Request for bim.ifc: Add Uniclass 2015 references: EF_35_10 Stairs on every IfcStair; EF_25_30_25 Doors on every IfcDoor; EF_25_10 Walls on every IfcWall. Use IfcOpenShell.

First a look at what the model holds.

```python
import ifcopenshell

model = ifcopenshell.open("bim.ifc")
print(model.schema)
print("classifications:", [c.Name for c in model.by_type("IfcClassification")])
for ifc_class in ("IfcDoor", "IfcRoof", "IfcStair", "IfcWall", "IfcWindow"):
    print(ifc_class, len(model.by_type(ifc_class)))
```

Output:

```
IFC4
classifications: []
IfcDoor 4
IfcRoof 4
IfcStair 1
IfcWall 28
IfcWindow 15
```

```python
import ifcopenshell
import ifcopenshell.api.classification

model = ifcopenshell.open("bim.ifc")

system = ifcopenshell.api.classification.add_classification(model, classification="Uniclass 2015")

codes = {
    "IfcStair": ("EF_35_10", "Stairs"),
    "IfcDoor": ("EF_25_30_25", "Doors"),
    "IfcWall": ("EF_25_10", "Walls"),
}
for ifc_class, (code, name) in codes.items():
    products = model.by_type(ifc_class)
    ifcopenshell.api.classification.add_reference(
        model, products=products, classification=system, identification=code, name=name
    )
    print(code, len(products))

model.write("bim_v2.ifc")
```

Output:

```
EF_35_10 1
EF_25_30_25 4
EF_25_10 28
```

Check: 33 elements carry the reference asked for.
